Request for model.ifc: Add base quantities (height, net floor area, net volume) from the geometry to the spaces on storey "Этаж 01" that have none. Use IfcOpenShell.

First a look at what the model holds.

```python
import ifcopenshell
import ifcopenshell.util.element
import ifcopenshell.util.unit

model = ifcopenshell.open("model.ifc")
print(model.schema)
for unit_type in ("LENGTHUNIT", "AREAUNIT", "VOLUMEUNIT"):
    print(unit_type, ifcopenshell.util.unit.calculate_unit_scale(model, unit_type))
storey = next(s for s in model.by_type("IfcBuildingStorey") if s.Name == "Этаж 01")
spaces = [e for e in ifcopenshell.util.element.get_decomposition(storey) if e.is_a("IfcSpace")]
for e in sorted(spaces, key=lambda e: e.id()):
    print(e.id(), e.is_a(), e.Name, list(ifcopenshell.util.element.get_psets(e, qtos_only=True)), sep=" | ")
```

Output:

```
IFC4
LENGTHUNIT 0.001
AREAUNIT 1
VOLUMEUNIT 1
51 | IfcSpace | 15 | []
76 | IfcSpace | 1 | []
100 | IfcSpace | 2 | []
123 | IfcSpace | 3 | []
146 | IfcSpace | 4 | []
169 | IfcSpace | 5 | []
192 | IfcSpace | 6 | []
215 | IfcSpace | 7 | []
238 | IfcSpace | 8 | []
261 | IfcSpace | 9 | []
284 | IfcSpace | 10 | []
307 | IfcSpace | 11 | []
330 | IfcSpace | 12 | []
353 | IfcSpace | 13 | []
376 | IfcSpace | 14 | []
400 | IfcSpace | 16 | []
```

```python
import ifcopenshell
import ifcopenshell.api.pset
import ifcopenshell.geom
import ifcopenshell.util.element
import ifcopenshell.util.shape
import ifcopenshell.util.unit

model = ifcopenshell.open("model.ifc")
unit_scale = ifcopenshell.util.unit.calculate_unit_scale(model)
area_scale = ifcopenshell.util.unit.calculate_unit_scale(model, "AREAUNIT")
volume_scale = ifcopenshell.util.unit.calculate_unit_scale(model, "VOLUMEUNIT")
settings = ifcopenshell.geom.settings()

storey = next(s for s in model.by_type("IfcBuildingStorey") if s.Name == "Этаж 01")
spaces = [e for e in ifcopenshell.util.element.get_decomposition(storey) if e.is_a("IfcSpace")]

for e in sorted(spaces, key=lambda e: e.id()):
    if ifcopenshell.util.element.get_psets(e, qtos_only=True, should_inherit=False):
        continue
    # Geometry comes back in metres, in the element's own axes.
    shape = ifcopenshell.geom.create_shape(settings, e)
    values = {
        "Height": ifcopenshell.util.shape.get_z(shape.geometry) / unit_scale,
        "NetFloorArea": ifcopenshell.util.shape.get_footprint_area(shape.geometry) / area_scale,
        "NetVolume": ifcopenshell.util.shape.get_volume(shape.geometry) / volume_scale,
    }
    qto = ifcopenshell.api.pset.add_qto(model, product=e, name="Qto_SpaceBaseQuantities")
    ifcopenshell.api.pset.edit_qto(model, qto=qto, properties=values)
    print(e.id(), {k: round(v, 3) for k, v in values.items()})

model.write("model_rev.ifc")
```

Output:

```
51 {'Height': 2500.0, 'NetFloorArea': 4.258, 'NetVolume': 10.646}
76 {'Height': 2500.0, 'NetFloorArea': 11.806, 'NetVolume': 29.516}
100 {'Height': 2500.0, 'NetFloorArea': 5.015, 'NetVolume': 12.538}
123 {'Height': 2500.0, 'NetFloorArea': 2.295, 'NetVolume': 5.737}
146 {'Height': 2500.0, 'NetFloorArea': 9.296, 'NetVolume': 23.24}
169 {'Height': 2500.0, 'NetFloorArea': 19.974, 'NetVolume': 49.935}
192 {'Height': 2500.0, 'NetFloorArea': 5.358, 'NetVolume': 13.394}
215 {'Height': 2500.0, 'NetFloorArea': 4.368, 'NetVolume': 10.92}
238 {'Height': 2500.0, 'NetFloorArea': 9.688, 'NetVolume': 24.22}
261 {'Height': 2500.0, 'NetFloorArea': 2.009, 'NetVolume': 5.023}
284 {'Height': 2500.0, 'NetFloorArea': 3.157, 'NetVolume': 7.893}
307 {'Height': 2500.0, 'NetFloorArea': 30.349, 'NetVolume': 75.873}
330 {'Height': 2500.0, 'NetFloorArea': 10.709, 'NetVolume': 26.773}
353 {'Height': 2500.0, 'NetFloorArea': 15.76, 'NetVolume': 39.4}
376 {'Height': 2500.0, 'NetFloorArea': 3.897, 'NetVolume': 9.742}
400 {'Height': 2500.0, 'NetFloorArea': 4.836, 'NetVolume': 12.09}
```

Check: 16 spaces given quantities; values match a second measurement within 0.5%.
